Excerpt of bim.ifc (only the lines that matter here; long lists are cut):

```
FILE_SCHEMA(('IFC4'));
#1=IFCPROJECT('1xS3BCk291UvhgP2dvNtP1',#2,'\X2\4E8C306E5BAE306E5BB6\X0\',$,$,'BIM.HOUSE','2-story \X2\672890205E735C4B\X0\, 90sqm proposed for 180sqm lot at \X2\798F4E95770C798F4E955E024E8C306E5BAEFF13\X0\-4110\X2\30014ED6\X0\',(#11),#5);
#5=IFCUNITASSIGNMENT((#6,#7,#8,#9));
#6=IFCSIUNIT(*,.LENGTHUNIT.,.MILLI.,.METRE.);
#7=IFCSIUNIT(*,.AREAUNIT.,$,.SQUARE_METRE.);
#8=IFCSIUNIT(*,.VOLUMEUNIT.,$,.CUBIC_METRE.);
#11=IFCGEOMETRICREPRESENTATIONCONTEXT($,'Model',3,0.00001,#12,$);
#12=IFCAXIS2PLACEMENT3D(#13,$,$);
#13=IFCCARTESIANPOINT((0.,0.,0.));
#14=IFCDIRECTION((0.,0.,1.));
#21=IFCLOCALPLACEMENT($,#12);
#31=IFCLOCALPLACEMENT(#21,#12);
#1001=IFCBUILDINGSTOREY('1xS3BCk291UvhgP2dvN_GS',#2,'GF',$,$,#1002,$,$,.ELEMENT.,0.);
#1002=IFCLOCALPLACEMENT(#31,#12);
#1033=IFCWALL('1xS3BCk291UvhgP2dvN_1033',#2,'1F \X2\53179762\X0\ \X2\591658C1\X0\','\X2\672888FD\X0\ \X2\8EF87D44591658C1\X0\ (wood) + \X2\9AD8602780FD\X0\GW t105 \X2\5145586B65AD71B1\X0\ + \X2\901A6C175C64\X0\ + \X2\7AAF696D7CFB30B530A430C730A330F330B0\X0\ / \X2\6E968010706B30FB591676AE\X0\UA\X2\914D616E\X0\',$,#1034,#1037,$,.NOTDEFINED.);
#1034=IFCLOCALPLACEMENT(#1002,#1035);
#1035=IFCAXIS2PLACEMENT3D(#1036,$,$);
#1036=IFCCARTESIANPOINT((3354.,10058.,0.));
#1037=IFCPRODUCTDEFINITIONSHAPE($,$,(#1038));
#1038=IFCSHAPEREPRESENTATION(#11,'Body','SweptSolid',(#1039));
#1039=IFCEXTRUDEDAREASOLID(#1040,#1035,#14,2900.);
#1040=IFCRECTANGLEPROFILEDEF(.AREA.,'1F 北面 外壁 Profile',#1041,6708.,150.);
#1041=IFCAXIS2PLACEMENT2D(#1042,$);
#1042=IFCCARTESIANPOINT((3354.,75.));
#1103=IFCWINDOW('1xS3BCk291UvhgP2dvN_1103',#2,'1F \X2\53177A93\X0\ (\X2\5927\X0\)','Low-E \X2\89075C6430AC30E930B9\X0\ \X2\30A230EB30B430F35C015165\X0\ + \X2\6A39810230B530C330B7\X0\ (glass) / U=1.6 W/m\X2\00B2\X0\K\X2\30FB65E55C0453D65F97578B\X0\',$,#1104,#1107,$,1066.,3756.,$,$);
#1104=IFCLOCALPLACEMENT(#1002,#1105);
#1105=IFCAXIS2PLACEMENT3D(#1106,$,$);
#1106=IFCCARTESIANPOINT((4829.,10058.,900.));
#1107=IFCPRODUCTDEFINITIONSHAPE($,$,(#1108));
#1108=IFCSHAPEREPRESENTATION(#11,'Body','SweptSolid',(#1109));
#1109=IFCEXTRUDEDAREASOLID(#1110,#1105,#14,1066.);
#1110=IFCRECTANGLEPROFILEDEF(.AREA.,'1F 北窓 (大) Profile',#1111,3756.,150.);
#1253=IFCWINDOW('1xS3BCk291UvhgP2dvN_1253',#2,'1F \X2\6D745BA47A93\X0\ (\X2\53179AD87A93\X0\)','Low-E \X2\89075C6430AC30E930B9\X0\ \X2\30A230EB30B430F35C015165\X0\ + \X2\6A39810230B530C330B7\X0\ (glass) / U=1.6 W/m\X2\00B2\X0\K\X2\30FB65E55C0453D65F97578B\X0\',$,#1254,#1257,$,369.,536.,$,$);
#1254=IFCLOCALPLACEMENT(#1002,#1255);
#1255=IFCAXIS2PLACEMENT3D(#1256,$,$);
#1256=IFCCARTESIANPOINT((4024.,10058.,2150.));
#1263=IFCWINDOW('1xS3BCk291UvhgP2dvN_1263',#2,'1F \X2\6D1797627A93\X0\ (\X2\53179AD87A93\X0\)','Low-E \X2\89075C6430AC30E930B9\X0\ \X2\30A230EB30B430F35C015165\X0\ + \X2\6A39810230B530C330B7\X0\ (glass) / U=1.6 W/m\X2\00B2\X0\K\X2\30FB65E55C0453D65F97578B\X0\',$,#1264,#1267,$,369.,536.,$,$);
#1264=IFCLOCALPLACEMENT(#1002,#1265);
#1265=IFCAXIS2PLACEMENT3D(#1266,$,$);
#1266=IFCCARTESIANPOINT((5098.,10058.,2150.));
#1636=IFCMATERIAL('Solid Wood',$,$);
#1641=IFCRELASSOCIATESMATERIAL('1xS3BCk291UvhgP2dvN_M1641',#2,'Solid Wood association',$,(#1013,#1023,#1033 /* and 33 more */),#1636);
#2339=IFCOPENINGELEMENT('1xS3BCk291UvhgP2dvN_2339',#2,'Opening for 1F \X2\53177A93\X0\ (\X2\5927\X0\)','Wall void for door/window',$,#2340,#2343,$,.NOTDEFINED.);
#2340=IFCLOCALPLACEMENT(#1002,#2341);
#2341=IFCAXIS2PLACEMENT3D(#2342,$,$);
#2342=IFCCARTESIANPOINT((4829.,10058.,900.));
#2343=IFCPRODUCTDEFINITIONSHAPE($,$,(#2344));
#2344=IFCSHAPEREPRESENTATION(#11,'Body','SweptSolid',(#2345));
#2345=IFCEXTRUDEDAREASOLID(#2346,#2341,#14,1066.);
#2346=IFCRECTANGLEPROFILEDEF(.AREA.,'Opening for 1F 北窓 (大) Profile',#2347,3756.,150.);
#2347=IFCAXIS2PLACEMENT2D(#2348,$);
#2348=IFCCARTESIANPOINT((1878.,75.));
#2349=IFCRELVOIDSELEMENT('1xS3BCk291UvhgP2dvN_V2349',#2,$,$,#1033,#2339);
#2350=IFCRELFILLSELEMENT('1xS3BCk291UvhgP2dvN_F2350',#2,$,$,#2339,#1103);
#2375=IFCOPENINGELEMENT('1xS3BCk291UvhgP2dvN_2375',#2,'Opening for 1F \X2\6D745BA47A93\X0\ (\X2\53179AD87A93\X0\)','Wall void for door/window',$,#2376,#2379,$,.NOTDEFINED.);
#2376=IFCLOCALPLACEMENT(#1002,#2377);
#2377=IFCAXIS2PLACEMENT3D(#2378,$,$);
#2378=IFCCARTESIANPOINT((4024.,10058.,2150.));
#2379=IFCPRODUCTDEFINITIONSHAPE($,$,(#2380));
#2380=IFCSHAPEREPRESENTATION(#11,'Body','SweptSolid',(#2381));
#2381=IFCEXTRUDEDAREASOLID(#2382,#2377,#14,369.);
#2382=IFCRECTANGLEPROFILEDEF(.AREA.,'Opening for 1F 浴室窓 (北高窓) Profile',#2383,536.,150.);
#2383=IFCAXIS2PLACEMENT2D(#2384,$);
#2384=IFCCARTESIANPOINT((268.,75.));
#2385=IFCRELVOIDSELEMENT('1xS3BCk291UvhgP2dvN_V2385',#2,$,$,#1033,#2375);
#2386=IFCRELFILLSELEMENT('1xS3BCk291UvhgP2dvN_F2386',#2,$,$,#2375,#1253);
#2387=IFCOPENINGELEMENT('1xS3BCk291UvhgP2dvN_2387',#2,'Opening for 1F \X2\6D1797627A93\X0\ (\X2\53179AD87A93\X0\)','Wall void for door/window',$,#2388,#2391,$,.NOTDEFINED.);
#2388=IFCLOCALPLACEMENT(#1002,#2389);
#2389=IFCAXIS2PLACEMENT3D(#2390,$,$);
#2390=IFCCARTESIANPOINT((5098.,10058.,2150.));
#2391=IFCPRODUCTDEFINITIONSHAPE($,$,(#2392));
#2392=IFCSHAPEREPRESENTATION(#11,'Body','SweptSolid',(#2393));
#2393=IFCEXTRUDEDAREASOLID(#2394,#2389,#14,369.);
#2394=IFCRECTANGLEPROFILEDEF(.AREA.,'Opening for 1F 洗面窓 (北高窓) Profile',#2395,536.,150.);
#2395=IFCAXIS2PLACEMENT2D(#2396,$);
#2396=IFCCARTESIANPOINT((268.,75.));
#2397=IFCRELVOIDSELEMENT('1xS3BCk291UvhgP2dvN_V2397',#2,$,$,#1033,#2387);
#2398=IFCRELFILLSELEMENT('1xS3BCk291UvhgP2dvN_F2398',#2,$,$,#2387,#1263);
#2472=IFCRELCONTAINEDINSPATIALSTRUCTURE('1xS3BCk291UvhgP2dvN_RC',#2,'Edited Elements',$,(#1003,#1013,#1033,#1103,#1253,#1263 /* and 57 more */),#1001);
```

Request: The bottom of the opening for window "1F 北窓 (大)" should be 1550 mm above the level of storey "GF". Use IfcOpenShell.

```python
import numpy as np
import ifcopenshell
import ifcopenshell.api.geometry
import ifcopenshell.geom
import ifcopenshell.util.element
import ifcopenshell.util.placement
import ifcopenshell.util.shape
import ifcopenshell.util.unit

model = ifcopenshell.open("bim.ifc")
unit_scale = ifcopenshell.util.unit.calculate_unit_scale(model)

window = model.by_guid("1xS3BCk291UvhgP2dvN_1103")
opening = window.FillsVoids[0].RelatingOpeningElement
storey = ifcopenshell.util.element.get_container(window, ifc_class="IfcBuildingStorey")
level = ifcopenshell.util.placement.get_local_placement(storey.ObjectPlacement)[2, 3]

# The opening's origin need not be at the sill, so measure its lowest point.
shape = ifcopenshell.geom.create_shape(ifcopenshell.geom.settings(), opening)
bottom = ifcopenshell.util.shape.get_shape_bottom_elevation(shape, shape.geometry) / unit_scale
dz = level + 1.55 / unit_scale - bottom

shift = np.array([0.0, 0.0, dz])
# The window is not placed relative to its opening, so move both.
for product in (opening, window):
    matrix = ifcopenshell.util.placement.get_local_placement(product.ObjectPlacement)
    matrix[:3, 3] += shift
    ifcopenshell.api.geometry.edit_object_placement(model, product=product, matrix=matrix, is_si=False)

print(f"moved by {dz * unit_scale:+.3f} m")

model.write("bim_updated.ifc")
```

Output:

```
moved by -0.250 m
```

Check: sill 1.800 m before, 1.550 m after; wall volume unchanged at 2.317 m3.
